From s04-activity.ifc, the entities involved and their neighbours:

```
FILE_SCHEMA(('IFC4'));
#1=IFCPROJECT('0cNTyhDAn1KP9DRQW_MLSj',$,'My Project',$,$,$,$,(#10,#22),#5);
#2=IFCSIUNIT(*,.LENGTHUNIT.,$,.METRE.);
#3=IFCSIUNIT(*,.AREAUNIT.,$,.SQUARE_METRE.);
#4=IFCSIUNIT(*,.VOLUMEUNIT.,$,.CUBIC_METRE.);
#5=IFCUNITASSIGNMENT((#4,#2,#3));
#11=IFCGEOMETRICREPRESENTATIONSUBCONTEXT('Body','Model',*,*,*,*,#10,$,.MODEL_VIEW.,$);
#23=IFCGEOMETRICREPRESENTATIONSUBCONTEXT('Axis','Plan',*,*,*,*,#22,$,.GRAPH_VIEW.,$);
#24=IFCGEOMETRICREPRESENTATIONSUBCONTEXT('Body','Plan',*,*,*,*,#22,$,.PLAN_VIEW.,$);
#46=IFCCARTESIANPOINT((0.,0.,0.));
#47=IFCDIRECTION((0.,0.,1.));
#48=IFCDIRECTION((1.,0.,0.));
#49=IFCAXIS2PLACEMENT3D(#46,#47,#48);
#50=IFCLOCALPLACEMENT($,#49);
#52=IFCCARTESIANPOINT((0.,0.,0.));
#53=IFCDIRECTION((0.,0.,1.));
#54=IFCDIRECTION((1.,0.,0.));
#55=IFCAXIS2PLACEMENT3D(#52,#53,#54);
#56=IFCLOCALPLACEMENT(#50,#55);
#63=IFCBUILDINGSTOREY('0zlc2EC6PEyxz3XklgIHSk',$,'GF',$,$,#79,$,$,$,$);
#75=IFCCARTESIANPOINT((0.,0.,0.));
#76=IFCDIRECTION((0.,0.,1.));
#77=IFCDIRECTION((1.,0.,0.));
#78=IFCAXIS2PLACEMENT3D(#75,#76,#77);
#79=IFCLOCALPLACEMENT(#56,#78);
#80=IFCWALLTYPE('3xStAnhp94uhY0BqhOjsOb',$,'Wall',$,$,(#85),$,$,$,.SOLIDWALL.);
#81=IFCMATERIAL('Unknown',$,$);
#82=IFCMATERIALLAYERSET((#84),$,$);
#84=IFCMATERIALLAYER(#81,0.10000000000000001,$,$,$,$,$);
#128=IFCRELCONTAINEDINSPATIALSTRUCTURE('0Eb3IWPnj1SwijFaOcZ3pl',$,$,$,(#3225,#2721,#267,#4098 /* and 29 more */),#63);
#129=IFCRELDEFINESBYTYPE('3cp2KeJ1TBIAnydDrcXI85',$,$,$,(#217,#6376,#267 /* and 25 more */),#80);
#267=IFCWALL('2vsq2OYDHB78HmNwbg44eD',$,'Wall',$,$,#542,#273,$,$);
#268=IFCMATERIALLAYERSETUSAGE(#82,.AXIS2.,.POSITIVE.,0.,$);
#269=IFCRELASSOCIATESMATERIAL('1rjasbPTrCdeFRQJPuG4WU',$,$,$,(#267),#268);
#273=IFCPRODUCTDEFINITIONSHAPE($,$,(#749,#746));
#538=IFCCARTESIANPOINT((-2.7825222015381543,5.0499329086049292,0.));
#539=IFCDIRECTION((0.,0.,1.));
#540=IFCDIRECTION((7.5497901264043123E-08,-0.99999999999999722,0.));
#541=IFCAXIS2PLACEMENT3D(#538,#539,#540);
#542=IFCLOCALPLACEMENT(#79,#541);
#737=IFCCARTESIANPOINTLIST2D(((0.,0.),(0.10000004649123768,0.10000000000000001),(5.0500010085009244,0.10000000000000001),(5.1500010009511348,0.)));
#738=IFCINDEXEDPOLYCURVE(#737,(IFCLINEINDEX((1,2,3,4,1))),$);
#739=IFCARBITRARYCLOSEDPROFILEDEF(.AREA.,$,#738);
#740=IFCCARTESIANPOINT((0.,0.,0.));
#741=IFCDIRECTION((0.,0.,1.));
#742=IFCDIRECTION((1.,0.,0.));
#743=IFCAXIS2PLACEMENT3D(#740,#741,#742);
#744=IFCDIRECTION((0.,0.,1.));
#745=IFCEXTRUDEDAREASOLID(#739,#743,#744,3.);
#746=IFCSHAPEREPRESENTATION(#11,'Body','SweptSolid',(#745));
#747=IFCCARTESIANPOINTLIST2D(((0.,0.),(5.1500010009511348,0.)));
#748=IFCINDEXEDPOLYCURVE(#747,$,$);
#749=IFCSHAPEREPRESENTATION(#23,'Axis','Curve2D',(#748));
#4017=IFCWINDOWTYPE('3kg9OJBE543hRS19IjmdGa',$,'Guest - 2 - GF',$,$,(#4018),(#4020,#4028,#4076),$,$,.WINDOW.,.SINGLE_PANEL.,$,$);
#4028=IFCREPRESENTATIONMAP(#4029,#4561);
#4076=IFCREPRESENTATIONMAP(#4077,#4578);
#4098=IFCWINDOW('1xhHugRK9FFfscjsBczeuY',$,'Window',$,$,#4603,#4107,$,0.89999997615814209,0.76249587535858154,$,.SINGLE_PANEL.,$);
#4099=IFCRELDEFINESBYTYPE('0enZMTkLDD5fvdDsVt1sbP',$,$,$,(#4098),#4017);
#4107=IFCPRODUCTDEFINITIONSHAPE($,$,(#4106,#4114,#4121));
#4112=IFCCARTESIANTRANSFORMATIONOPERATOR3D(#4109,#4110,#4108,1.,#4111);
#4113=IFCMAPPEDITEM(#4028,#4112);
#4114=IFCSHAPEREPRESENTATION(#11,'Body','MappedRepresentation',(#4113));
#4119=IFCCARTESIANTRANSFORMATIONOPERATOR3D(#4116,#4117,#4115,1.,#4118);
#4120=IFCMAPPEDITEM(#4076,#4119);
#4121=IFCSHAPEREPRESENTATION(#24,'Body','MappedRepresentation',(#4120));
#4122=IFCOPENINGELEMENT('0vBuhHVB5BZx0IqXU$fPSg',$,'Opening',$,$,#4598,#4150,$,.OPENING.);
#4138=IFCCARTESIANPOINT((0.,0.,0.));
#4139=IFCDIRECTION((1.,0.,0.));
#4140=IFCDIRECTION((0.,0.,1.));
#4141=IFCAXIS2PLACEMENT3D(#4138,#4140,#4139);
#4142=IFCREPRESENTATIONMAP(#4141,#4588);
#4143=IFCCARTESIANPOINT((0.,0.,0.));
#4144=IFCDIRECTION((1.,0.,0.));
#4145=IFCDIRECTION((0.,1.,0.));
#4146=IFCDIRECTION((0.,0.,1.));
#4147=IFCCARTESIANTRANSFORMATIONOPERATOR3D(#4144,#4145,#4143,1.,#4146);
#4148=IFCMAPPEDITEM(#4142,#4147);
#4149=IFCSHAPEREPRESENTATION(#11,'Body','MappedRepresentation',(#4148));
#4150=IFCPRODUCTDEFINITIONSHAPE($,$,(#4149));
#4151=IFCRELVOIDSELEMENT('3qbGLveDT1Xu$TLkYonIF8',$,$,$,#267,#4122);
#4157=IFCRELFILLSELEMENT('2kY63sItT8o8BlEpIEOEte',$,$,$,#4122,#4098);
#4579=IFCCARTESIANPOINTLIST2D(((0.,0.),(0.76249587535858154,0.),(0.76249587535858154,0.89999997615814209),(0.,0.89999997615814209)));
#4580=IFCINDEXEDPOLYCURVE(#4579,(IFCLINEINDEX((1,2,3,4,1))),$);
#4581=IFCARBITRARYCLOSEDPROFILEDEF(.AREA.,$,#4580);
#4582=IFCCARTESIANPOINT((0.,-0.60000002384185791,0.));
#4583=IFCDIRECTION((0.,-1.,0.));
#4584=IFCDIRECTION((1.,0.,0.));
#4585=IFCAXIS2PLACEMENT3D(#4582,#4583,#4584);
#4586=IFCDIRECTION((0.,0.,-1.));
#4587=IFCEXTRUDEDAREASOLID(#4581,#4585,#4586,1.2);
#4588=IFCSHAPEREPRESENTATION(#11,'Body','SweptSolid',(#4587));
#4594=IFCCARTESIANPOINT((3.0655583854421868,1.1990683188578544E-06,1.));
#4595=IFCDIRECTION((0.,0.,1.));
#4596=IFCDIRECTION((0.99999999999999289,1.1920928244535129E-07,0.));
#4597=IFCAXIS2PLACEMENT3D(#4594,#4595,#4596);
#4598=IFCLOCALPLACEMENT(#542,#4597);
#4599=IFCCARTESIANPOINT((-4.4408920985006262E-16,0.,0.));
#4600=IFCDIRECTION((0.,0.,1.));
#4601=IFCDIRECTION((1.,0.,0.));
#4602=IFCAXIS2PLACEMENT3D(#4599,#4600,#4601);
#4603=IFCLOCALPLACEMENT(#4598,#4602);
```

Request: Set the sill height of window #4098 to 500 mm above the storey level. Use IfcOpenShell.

```python
import numpy as np
import ifcopenshell
import ifcopenshell.api.geometry
import ifcopenshell.geom
import ifcopenshell.util.element
import ifcopenshell.util.placement
import ifcopenshell.util.shape
import ifcopenshell.util.unit

model = ifcopenshell.open("s04-activity.ifc")
unit_scale = ifcopenshell.util.unit.calculate_unit_scale(model)

window = model.by_id(4098)
opening = window.FillsVoids[0].RelatingOpeningElement
storey = ifcopenshell.util.element.get_container(window, ifc_class="IfcBuildingStorey")
level = ifcopenshell.util.placement.get_local_placement(storey.ObjectPlacement)[2, 3]

# The opening's origin need not be at the sill, so measure its lowest point.
shape = ifcopenshell.geom.create_shape(ifcopenshell.geom.settings(), opening)
bottom = ifcopenshell.util.shape.get_shape_bottom_elevation(shape, shape.geometry) / unit_scale
dz = level + 0.5 / unit_scale - bottom

shift = np.array([0.0, 0.0, dz])
# The window is placed relative to its opening, so it follows when the opening moves.
matrix = ifcopenshell.util.placement.get_local_placement(opening.ObjectPlacement)
matrix[:3, 3] += shift
ifcopenshell.api.geometry.edit_object_placement(
    model, product=opening, matrix=matrix, is_si=False, should_transform_children=True
)

print(f"moved by {dz * unit_scale:+.3f} m")

model.write("s04-activity_v2.ifc")
```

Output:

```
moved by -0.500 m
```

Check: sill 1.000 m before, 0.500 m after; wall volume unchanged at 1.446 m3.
